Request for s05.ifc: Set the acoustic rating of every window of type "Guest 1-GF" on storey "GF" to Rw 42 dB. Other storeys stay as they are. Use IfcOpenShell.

First a look at what the model holds.

```python
import ifcopenshell
import ifcopenshell.util.element

model = ifcopenshell.open("s05.ifc")
print(model.schema)
storey = next(s for s in model.by_type("IfcBuildingStorey") if s.Name == "GF")
windows = [e for e in ifcopenshell.util.element.get_decomposition(storey) if e.is_a("IfcWindow")]
seen = {}
for e in windows:
    element_type = ifcopenshell.util.element.get_type(e)
    key = (element_type.Name if element_type != e and element_type else None, ifcopenshell.util.element.get_pset(e, "Pset_WindowCommon", "AcousticRating"))
    seen[key] = seen.get(key, 0) + 1
for (name, value), count in sorted(seen.items(), key=str):
    print(count, "x", name, "|", value)
```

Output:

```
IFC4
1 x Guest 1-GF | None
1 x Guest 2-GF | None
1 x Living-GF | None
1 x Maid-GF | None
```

```python
import ifcopenshell
import ifcopenshell.api.pset
import ifcopenshell.util.element

model = ifcopenshell.open("s05.ifc")

storey = next(s for s in model.by_type("IfcBuildingStorey") if s.Name == "GF")
windows = [e for e in ifcopenshell.util.element.get_decomposition(storey) if e.is_a("IfcWindow")]

count = 0
for e in windows:
    element_type = ifcopenshell.util.element.get_type(e)
    if element_type in (None, e) or element_type.Name != "Guest 1-GF":
        continue
    # add_pset returns the element's existing set when there is one.
    pset = ifcopenshell.api.pset.add_pset(model, product=e, name="Pset_WindowCommon")
    ifcopenshell.api.pset.edit_pset(model, pset=pset, properties={"AcousticRating": "Rw 42 dB"})
    count += 1

print(count, "windows updated")

model.write("s05_updated.ifc")
```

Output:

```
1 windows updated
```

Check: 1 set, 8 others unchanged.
